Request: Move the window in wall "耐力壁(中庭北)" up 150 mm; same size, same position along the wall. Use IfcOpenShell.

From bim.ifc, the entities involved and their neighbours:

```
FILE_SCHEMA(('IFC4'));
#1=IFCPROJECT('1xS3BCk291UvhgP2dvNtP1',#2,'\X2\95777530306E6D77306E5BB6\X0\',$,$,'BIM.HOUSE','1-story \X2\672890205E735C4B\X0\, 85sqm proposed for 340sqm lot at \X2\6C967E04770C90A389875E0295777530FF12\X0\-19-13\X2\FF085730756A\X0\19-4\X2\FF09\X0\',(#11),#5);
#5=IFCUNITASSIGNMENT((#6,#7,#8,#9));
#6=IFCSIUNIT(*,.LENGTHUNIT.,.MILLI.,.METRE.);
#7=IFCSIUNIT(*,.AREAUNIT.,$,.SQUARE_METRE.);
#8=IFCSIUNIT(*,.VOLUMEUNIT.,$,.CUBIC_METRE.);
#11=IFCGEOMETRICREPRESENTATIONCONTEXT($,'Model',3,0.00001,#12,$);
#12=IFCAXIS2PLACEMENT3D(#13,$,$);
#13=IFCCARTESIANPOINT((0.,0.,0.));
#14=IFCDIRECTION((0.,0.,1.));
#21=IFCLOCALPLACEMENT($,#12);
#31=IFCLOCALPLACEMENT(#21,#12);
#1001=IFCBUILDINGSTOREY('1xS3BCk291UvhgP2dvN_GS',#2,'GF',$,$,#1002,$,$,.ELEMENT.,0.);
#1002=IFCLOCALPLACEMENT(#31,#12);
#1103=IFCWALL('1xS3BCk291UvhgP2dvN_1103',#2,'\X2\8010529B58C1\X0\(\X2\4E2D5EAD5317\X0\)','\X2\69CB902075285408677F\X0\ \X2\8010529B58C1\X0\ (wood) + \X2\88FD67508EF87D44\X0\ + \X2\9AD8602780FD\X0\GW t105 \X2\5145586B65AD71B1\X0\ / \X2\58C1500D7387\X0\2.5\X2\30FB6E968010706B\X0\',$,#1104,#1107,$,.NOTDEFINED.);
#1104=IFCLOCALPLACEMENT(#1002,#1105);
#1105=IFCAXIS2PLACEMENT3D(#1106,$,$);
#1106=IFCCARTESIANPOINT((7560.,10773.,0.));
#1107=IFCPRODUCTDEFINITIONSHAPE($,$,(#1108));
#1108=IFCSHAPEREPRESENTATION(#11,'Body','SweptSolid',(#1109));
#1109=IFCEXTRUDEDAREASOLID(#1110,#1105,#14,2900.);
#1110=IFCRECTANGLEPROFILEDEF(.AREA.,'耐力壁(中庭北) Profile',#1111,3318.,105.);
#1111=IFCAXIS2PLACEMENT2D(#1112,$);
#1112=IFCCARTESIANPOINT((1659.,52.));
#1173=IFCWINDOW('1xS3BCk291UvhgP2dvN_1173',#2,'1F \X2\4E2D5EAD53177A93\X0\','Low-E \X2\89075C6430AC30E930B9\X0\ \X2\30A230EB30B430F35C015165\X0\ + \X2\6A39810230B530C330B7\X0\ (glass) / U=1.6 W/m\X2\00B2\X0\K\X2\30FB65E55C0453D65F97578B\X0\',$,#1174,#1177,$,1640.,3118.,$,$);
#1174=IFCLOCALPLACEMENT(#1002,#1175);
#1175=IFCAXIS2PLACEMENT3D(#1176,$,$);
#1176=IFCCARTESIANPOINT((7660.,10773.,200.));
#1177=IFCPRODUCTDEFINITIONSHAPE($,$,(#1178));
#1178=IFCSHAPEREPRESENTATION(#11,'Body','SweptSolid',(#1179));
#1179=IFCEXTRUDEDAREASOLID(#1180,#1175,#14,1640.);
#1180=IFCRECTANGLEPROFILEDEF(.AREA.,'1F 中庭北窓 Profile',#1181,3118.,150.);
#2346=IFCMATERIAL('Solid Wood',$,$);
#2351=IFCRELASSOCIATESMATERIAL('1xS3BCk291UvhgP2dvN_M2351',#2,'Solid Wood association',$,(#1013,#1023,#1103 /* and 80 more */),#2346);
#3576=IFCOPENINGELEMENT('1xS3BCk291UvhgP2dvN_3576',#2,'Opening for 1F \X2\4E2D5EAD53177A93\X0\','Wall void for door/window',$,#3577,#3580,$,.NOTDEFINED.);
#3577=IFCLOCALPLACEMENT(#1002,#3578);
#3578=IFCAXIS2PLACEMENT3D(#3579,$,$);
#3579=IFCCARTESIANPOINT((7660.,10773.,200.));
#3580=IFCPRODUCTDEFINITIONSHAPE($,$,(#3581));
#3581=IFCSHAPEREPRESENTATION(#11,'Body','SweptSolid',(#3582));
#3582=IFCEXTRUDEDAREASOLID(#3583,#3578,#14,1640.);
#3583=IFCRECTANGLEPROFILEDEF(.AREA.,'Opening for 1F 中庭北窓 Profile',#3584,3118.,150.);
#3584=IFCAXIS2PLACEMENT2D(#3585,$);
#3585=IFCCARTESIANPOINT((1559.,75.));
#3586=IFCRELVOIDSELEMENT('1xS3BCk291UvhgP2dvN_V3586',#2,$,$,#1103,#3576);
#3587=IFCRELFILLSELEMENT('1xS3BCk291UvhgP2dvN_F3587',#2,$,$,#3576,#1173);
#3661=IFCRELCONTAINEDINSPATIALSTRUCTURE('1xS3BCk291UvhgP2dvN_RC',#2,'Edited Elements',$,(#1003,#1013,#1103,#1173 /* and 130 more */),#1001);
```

```python
import numpy as np
import ifcopenshell
import ifcopenshell.api.geometry
import ifcopenshell.util.placement
import ifcopenshell.util.unit

model = ifcopenshell.open("bim.ifc")
unit_scale = ifcopenshell.util.unit.calculate_unit_scale(model)

window = model.by_id(1173)
opening = window.FillsVoids[0].RelatingOpeningElement
dz = 0.15 / unit_scale

shift = np.array([0.0, 0.0, dz])
# The window is not placed relative to its opening, so move both.
for product in (opening, window):
    matrix = ifcopenshell.util.placement.get_local_placement(product.ObjectPlacement)
    matrix[:3, 3] += shift
    ifcopenshell.api.geometry.edit_object_placement(model, product=product, matrix=matrix, is_si=False)

print(f"moved by {dz * unit_scale:+.3f} m")

model.write("bim_updated.ifc")
```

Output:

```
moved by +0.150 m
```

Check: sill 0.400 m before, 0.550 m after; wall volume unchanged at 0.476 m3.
